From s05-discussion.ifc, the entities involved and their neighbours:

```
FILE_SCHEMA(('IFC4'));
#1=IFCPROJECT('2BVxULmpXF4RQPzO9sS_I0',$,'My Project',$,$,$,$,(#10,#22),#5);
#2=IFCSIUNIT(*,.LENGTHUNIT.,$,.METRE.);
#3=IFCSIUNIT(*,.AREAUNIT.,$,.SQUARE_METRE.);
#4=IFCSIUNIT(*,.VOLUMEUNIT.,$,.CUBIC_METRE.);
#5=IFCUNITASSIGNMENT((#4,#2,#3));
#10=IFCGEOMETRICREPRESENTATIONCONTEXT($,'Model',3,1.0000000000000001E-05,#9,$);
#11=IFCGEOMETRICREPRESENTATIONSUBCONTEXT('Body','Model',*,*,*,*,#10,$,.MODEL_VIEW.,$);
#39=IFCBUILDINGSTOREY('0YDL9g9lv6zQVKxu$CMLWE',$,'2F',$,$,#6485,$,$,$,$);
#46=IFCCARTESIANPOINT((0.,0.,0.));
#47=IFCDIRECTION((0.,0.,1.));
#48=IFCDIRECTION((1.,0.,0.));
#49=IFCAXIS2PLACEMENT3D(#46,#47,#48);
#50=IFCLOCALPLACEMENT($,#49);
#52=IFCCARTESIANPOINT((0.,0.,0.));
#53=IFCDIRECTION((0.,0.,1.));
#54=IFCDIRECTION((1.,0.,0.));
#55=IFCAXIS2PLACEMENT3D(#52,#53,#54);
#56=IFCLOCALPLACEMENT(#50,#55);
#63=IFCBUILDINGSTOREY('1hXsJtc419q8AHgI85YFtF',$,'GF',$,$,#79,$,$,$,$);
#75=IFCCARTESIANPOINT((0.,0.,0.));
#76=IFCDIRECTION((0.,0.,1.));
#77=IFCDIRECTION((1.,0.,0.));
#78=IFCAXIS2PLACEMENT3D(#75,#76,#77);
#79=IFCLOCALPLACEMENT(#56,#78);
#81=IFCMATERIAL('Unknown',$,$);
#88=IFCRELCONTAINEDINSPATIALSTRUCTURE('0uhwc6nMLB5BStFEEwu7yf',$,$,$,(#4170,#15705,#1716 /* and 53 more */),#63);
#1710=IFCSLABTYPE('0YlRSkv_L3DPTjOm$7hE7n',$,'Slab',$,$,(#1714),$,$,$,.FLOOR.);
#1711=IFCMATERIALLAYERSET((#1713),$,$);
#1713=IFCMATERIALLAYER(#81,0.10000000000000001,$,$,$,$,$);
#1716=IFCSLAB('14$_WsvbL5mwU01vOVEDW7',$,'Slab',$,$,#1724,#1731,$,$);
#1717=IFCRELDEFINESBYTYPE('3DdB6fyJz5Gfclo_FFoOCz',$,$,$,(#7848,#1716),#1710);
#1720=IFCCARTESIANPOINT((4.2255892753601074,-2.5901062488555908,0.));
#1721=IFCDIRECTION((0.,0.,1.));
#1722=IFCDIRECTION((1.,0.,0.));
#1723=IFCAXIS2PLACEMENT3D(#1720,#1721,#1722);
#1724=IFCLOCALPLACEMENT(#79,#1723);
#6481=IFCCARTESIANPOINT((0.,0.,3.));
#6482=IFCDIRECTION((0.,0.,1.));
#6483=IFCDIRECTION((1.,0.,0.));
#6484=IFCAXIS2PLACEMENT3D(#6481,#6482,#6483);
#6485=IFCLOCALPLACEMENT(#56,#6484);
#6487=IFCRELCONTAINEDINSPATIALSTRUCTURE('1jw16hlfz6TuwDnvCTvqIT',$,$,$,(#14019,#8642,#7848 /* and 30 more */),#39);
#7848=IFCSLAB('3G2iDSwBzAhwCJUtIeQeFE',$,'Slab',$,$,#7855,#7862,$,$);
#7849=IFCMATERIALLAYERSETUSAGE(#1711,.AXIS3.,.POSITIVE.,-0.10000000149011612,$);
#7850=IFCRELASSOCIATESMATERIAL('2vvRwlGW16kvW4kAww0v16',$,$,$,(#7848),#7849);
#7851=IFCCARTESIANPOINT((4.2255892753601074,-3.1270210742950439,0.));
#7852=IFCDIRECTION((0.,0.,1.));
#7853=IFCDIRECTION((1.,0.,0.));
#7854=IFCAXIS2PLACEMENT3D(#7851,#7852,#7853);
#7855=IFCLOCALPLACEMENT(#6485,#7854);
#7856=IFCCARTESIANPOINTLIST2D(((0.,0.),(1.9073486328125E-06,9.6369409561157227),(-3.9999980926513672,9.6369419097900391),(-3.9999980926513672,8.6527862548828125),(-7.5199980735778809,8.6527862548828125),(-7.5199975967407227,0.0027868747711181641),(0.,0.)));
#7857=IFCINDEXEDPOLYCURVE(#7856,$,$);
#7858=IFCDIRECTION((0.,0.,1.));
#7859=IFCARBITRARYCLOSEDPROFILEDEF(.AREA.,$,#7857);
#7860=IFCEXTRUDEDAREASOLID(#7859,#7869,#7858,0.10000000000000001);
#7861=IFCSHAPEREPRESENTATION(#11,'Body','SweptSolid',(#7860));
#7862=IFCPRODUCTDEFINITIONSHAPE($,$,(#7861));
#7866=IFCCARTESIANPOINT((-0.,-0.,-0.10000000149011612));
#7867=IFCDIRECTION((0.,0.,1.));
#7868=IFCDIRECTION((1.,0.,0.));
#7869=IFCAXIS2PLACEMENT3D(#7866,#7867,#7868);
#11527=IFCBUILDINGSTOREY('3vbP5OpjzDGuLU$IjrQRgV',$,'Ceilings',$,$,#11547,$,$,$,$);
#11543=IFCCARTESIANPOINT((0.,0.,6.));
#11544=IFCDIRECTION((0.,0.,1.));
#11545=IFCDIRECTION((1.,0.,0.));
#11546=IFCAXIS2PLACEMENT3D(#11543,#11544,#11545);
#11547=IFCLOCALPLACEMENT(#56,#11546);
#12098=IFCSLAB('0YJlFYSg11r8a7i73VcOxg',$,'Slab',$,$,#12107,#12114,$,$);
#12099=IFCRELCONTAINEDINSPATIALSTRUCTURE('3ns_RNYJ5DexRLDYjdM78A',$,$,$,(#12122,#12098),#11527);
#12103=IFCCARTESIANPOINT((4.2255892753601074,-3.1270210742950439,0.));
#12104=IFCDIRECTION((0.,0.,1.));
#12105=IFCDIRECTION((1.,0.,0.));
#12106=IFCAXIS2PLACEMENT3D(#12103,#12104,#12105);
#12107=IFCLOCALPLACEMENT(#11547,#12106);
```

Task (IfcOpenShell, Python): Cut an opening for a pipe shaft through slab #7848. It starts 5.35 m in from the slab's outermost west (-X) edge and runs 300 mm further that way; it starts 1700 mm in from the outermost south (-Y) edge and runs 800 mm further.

```python
import numpy as np
import ifcopenshell
import ifcopenshell.api.feature
import ifcopenshell.api.geometry
import ifcopenshell.api.root
import ifcopenshell.geom
import ifcopenshell.util.placement
import ifcopenshell.util.representation
import ifcopenshell.util.shape
import ifcopenshell.util.unit

model = ifcopenshell.open("s05-discussion.ifc")
unit_scale = ifcopenshell.util.unit.calculate_unit_scale(model)
settings = ifcopenshell.geom.settings()


def volume(element):
    """Net volume in cubic metres, openings subtracted."""
    shape = ifcopenshell.geom.create_shape(settings, element)
    return ifcopenshell.util.shape.get_volume(shape.geometry)


slab = model.by_guid("3G2iDSwBzAhwCJUtIeQeFE")
before = volume(slab)

# Extent in the slab's own axes, in metres. The edges named are its -X and -Y sides.
slab_shape = ifcopenshell.geom.create_shape(settings, slab)
vertices = ifcopenshell.util.shape.get_vertices(slab_shape.geometry)
x_min, y_min, bottom = vertices.min(axis=0)
top = vertices[:, 2].max()

opening = ifcopenshell.api.root.create_entity(model, ifc_class="IfcOpeningElement", name="Pipe shaft opening", predefined_type="OPENING")
context = ifcopenshell.util.representation.get_context(model, "Model", "Body", "MODEL_VIEW")
width, depth = 0.3, 0.8
outline = [(0.0, 0.0), (width, 0.0), (width, depth), (0.0, depth), (0.0, 0.0)]
# Overshoot both faces by 50 mm so the cut is clean.
shape = ifcopenshell.api.geometry.add_slab_representation(
    model, context=context, depth=top - bottom + 0.1, polyline=outline
)
ifcopenshell.api.geometry.assign_representation(model, product=opening, representation=shape)

matrix = ifcopenshell.util.placement.get_local_placement(slab.ObjectPlacement)
matrix[:, 3] = matrix @ np.append(np.array([x_min + 5.35, y_min + 1.7, bottom - 0.05]) / unit_scale, 1.0)
ifcopenshell.api.geometry.edit_object_placement(model, product=opening, matrix=matrix, is_si=False)
ifcopenshell.api.feature.add_feature(model, feature=opening, element=slab)

after = volume(slab)

print(f"slab volume {before:.3f} -> {after:.3f} m3")

model.write("s05-discussion_updated.ifc")
```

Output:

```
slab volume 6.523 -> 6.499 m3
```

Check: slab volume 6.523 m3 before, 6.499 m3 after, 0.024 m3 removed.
